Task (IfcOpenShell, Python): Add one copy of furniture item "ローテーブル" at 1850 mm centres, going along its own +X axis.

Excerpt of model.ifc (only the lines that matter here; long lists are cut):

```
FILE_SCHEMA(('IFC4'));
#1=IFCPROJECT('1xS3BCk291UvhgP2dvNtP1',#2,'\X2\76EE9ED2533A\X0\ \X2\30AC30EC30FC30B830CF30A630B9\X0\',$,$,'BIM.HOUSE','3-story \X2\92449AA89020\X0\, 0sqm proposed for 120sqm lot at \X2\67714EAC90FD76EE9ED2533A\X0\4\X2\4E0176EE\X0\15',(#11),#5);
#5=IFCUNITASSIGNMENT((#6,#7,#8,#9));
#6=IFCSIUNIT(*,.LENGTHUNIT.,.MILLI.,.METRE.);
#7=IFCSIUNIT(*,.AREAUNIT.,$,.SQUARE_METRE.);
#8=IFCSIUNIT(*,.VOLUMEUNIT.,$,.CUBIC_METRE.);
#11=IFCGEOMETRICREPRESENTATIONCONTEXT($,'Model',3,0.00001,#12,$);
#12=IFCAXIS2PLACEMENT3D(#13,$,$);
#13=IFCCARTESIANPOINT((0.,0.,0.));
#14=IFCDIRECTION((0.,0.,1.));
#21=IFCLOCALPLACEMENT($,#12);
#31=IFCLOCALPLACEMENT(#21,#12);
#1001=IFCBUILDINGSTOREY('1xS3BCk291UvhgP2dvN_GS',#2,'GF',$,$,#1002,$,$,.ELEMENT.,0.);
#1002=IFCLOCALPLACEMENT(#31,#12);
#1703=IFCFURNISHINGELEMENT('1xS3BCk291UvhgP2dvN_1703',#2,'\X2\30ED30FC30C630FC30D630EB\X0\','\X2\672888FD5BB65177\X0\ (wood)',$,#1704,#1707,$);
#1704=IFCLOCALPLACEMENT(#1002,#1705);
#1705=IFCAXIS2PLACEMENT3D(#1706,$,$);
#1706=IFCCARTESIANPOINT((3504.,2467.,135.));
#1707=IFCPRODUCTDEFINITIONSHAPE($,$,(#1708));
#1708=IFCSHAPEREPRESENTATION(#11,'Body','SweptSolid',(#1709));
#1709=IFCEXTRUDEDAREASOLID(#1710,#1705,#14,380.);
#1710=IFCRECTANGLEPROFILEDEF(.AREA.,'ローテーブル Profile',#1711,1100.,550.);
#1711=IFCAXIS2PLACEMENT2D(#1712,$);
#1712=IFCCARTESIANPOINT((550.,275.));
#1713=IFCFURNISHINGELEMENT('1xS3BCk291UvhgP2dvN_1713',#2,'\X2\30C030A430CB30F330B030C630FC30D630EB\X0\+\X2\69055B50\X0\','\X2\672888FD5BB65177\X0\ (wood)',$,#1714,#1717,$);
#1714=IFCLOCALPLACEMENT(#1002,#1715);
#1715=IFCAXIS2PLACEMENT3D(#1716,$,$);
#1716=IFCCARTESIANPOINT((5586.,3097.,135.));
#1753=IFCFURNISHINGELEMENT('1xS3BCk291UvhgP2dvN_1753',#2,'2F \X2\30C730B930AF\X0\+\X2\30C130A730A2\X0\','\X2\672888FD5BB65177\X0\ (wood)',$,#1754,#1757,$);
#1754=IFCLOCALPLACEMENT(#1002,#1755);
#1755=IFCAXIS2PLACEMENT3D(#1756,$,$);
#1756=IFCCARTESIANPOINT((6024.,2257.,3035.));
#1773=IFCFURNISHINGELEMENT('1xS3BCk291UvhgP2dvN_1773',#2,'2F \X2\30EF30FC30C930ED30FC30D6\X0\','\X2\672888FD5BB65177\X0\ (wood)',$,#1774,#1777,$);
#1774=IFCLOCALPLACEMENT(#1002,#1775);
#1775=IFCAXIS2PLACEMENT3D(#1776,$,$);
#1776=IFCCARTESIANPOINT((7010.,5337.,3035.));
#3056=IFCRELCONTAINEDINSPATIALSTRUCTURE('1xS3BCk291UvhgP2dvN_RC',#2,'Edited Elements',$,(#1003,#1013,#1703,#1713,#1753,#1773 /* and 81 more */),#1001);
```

```python
import ifcopenshell
import ifcopenshell.api.geometry
import ifcopenshell.api.root
import ifcopenshell.util.element
import ifcopenshell.util.placement
import ifcopenshell.util.unit

model = ifcopenshell.open("model.ifc")
unit_scale = ifcopenshell.util.unit.calculate_unit_scale(model)


def reuse_history(source, copy):
    """copy_class also copies each property set's owner history, people and application; keep the originals."""
    for rel in copy.IsDefinedBy:
        if rel.is_a("IfcRelDefinesByProperties") and (history := rel.RelatingPropertyDefinition.OwnerHistory):
            rel.RelatingPropertyDefinition.OwnerHistory = source.OwnerHistory
            ifcopenshell.util.element.remove_deep2(model, history)


source = model.by_id(1703)
base = ifcopenshell.util.placement.get_local_placement(source.ObjectPlacement)
step = base[:3, 0] * 1.85 / unit_scale

for i in range(1, 2):
    copy = ifcopenshell.api.root.copy_class(model, product=source)
    copy.Representation = ifcopenshell.util.element.copy_deep(
        model, source.Representation, exclude=["IfcGeometricRepresentationContext", "IfcRepresentationMap"]
    )
    reuse_history(source, copy)
    matrix = base.copy()
    matrix[:3, 3] += i * step
    print("added at", matrix[:3, 3].round(3) + 0.0)
    ifcopenshell.api.geometry.edit_object_placement(model, product=copy, matrix=matrix, is_si=False)

model.write("model-out.ifc")
```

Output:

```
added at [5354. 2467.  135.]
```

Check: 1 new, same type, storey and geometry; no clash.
